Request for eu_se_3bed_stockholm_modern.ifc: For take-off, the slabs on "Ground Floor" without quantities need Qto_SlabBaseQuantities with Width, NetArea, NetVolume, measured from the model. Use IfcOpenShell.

First a look at what the model holds.

```python
import ifcopenshell
import ifcopenshell.util.element
import ifcopenshell.util.unit

model = ifcopenshell.open("eu_se_3bed_stockholm_modern.ifc")
print(model.schema)
for unit_type in ("LENGTHUNIT", "AREAUNIT", "VOLUMEUNIT"):
    print(unit_type, ifcopenshell.util.unit.calculate_unit_scale(model, unit_type))
storey = next(s for s in model.by_type("IfcBuildingStorey") if s.Name == "Ground Floor")
slabs = [e for e in ifcopenshell.util.element.get_decomposition(storey) if e.is_a("IfcSlab")]
for e in sorted(slabs, key=lambda e: e.id()):
    print(e.id(), e.is_a(), e.Name, list(ifcopenshell.util.element.get_psets(e, qtos_only=True)), sep=" | ")
```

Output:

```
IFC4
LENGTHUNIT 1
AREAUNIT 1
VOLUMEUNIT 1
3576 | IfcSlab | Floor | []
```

```python
import ifcopenshell
import ifcopenshell.api.pset
import ifcopenshell.geom
import ifcopenshell.util.element
import ifcopenshell.util.shape
import ifcopenshell.util.unit

model = ifcopenshell.open("eu_se_3bed_stockholm_modern.ifc")
unit_scale = ifcopenshell.util.unit.calculate_unit_scale(model)
area_scale = ifcopenshell.util.unit.calculate_unit_scale(model, "AREAUNIT")
volume_scale = ifcopenshell.util.unit.calculate_unit_scale(model, "VOLUMEUNIT")
settings = ifcopenshell.geom.settings()

storey = next(s for s in model.by_type("IfcBuildingStorey") if s.Name == "Ground Floor")
slabs = [e for e in ifcopenshell.util.element.get_decomposition(storey) if e.is_a("IfcSlab")]

for e in sorted(slabs, key=lambda e: e.id()):
    if ifcopenshell.util.element.get_psets(e, qtos_only=True, should_inherit=False):
        continue
    # Geometry comes back in metres, in the element's own axes.
    shape = ifcopenshell.geom.create_shape(settings, e)
    values = {
        "Width": ifcopenshell.util.shape.get_z(shape.geometry) / unit_scale,
        "NetArea": ifcopenshell.util.shape.get_footprint_area(shape.geometry) / area_scale,
        "NetVolume": ifcopenshell.util.shape.get_volume(shape.geometry) / volume_scale,
    }
    qto = ifcopenshell.api.pset.add_qto(model, product=e, name="Qto_SlabBaseQuantities")
    ifcopenshell.api.pset.edit_qto(model, qto=qto, properties=values)
    print(e.id(), {k: round(v, 3) for k, v in values.items()})

model.write("eu_se_3bed_stockholm_modern_edited.ifc")
```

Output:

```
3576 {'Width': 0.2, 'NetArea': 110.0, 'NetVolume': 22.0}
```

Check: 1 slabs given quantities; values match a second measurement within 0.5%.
